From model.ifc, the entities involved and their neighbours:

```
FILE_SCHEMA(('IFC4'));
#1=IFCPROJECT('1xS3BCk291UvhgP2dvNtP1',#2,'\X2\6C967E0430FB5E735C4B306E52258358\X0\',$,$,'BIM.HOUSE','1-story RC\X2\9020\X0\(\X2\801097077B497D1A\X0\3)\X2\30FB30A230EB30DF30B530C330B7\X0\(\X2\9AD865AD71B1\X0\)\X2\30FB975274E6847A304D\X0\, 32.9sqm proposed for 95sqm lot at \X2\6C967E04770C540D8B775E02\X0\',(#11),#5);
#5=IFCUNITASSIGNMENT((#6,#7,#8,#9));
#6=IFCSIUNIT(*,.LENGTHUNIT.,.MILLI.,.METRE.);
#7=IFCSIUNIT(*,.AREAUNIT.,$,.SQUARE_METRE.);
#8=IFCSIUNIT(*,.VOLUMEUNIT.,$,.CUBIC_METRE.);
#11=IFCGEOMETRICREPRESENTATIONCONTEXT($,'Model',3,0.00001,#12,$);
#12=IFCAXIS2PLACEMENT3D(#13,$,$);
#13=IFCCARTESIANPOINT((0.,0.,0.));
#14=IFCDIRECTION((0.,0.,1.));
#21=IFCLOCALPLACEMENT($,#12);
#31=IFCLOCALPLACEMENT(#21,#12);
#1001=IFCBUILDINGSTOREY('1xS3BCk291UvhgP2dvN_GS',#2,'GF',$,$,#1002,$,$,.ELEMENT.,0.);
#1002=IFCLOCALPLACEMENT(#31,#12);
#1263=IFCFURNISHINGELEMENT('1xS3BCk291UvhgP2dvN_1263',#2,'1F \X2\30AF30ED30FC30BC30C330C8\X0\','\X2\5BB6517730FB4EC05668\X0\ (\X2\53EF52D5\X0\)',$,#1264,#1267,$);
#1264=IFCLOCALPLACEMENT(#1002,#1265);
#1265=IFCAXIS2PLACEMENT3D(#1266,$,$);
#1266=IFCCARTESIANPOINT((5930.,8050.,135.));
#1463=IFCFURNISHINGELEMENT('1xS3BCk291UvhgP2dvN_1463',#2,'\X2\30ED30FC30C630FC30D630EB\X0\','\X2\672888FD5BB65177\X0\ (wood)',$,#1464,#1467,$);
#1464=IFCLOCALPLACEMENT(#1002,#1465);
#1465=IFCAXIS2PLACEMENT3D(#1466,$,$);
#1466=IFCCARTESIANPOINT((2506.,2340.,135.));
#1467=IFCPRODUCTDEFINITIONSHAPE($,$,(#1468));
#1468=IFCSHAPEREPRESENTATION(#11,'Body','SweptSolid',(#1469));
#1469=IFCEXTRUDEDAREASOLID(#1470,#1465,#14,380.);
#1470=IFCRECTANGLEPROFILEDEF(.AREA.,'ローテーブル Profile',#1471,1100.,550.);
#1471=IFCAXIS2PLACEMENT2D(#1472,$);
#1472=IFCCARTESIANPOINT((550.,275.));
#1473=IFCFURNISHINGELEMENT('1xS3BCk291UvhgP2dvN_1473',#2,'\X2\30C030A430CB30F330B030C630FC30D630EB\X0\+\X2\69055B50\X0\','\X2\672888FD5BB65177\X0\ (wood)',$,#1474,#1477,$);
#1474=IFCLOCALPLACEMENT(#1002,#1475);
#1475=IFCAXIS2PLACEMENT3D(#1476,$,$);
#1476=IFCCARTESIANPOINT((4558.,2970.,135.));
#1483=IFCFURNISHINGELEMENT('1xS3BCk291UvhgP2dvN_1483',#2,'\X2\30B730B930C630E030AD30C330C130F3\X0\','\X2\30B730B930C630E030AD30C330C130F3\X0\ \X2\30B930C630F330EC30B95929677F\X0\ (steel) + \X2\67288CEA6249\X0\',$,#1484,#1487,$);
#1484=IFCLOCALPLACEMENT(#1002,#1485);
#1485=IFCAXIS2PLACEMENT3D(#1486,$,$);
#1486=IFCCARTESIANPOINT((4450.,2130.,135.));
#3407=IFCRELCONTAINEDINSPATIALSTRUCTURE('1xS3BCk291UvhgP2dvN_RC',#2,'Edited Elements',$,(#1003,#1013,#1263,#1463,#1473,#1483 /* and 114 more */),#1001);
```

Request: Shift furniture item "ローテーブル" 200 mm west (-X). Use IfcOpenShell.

```python
import ifcopenshell
import ifcopenshell.api.geometry
import ifcopenshell.util.placement

model = ifcopenshell.open("model.ifc")

item = model.by_id(1463)
matrix = ifcopenshell.util.placement.get_local_placement(item.ObjectPlacement)
matrix[0, 3] -= 200.0
ifcopenshell.api.geometry.edit_object_placement(model, product=item, matrix=matrix, is_si=False)

print(ifcopenshell.util.placement.get_local_placement(item.ObjectPlacement).round(3) + 0.0)

model.write("model_rev.ifc")
```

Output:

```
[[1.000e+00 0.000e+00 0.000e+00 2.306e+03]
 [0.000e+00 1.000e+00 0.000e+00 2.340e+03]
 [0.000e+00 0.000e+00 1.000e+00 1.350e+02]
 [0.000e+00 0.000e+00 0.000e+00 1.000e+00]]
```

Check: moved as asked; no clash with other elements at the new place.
